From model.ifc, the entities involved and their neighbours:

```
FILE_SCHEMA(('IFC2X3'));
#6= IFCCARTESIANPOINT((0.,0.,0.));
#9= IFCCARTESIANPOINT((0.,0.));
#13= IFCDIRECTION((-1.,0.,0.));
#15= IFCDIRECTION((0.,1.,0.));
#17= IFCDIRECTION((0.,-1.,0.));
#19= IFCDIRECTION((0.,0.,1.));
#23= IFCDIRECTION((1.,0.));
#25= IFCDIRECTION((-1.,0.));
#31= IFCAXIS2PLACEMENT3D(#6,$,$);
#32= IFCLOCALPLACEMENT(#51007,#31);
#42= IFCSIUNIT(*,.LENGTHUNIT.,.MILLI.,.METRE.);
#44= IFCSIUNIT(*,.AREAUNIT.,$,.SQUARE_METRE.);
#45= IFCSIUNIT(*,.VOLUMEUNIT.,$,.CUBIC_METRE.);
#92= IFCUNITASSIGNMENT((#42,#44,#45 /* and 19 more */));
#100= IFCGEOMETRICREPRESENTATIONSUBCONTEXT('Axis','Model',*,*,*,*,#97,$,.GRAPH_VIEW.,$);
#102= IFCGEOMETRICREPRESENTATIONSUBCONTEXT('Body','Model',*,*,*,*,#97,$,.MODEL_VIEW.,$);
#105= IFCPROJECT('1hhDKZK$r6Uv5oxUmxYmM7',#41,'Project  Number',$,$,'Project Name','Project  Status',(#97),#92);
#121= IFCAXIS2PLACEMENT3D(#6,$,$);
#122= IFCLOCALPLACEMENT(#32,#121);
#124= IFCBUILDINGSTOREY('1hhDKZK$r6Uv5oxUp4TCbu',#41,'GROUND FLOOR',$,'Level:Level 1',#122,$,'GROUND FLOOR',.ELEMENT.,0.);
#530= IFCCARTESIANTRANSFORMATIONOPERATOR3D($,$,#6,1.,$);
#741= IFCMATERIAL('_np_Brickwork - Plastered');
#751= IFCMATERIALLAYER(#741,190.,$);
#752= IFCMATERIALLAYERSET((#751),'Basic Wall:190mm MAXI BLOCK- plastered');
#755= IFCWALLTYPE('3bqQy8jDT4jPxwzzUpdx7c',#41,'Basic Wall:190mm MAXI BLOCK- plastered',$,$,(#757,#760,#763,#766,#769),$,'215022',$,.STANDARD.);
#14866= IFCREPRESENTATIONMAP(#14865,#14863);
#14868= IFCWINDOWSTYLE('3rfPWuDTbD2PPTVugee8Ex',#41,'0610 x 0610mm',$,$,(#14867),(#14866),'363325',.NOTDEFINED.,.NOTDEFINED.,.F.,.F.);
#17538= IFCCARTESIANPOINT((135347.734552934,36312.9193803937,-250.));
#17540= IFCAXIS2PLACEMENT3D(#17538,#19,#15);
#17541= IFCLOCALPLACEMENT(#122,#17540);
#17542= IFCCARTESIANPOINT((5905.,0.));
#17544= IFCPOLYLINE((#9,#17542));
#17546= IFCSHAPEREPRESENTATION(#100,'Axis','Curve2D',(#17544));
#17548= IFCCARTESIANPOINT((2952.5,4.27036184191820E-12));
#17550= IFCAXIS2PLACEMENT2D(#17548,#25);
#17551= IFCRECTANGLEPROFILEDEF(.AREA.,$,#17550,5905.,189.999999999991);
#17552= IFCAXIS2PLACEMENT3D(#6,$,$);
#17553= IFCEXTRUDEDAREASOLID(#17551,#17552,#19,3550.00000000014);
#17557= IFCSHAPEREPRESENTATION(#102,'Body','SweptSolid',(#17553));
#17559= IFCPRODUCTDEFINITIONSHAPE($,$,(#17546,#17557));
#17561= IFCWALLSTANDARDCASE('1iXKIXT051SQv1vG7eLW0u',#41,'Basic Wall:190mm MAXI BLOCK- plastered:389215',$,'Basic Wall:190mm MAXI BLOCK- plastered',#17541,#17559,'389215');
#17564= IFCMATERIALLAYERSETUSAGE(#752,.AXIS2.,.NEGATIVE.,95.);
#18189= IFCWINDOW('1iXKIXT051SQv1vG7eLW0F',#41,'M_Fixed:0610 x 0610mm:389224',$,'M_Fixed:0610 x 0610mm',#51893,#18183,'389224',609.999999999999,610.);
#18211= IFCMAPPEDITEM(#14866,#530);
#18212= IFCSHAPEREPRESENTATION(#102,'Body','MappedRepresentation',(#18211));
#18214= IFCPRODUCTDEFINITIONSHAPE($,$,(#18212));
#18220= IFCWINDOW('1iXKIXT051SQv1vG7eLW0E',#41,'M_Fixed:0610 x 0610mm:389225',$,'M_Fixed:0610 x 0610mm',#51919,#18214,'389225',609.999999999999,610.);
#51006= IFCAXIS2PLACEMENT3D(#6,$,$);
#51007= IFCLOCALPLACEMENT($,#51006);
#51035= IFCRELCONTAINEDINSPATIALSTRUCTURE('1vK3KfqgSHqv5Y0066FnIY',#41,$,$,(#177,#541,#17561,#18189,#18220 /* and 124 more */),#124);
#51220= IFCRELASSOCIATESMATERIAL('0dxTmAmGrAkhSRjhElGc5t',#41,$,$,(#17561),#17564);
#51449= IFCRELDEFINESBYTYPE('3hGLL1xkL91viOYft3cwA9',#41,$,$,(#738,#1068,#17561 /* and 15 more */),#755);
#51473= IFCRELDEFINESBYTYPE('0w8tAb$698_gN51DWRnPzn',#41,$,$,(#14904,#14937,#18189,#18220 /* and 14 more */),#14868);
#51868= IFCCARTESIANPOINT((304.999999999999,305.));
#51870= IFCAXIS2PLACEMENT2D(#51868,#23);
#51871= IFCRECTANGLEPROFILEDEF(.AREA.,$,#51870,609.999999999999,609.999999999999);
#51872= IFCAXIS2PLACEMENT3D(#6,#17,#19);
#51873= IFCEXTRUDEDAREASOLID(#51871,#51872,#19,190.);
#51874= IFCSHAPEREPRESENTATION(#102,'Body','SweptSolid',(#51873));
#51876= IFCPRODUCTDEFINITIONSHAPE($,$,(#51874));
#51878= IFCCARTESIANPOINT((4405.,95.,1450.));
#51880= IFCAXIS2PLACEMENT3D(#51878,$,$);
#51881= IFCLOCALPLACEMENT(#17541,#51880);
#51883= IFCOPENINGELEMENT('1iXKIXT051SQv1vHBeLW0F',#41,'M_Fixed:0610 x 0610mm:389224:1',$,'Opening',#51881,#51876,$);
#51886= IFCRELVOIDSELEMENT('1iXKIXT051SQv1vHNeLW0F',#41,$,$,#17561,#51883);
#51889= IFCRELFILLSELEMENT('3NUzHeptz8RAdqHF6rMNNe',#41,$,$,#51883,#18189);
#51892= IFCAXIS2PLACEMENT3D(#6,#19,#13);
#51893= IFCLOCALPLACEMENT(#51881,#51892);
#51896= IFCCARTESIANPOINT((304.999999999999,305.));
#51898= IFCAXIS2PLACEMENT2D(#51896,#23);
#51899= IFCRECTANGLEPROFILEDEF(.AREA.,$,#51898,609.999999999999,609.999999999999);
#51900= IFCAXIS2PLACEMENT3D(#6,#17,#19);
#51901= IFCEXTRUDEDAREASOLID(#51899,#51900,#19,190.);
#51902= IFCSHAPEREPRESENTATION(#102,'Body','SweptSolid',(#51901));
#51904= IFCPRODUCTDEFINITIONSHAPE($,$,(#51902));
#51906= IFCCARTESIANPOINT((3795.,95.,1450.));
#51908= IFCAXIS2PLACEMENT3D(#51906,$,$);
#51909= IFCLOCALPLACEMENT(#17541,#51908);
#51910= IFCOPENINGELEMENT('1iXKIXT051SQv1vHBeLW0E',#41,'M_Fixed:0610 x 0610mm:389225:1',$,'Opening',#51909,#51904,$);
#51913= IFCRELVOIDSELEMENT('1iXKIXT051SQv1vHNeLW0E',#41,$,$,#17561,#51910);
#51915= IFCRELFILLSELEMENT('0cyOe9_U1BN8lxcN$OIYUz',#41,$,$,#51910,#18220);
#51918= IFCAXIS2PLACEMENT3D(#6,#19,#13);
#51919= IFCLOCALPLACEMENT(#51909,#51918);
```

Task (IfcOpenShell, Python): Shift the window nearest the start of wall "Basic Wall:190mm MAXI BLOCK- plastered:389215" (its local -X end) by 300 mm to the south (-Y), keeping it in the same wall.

```python
import ifcopenshell
import ifcopenshell.api.geometry
import ifcopenshell.util.placement
import ifcopenshell.util.unit

model = ifcopenshell.open("model.ifc")
unit_scale = ifcopenshell.util.unit.calculate_unit_scale(model)

window = model.by_id(18220)
opening = window.FillsVoids[0].RelatingOpeningElement
wall = opening.VoidsElements[0].RelatingBuildingElement

wall_matrix = ifcopenshell.util.placement.get_local_placement(wall.ObjectPlacement)
shift = wall_matrix[:3, 0] * -0.3 / unit_scale
before = ifcopenshell.util.placement.get_local_placement(window.ObjectPlacement)[:3, 3].copy()

# The window is placed relative to its opening, so it follows when the opening moves.
matrix = ifcopenshell.util.placement.get_local_placement(opening.ObjectPlacement)
matrix[:3, 3] += shift
ifcopenshell.api.geometry.edit_object_placement(
    model, product=opening, matrix=matrix, is_si=False, should_transform_children=True
)

after = ifcopenshell.util.placement.get_local_placement(window.ObjectPlacement)[:3, 3]
print("window moved by", (after - before).round(3) + 0.0)

model.write("model_edited.ifc")
```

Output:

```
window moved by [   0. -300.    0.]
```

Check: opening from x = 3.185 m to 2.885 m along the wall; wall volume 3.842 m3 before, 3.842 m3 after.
